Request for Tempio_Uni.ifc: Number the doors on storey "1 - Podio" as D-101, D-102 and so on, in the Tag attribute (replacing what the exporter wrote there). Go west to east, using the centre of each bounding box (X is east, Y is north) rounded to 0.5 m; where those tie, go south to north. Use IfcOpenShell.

First a look at what the model holds.

```python
import ifcopenshell
import ifcopenshell.util.element
import ifcopenshell.util.placement

model = ifcopenshell.open("Tempio_Uni.ifc")
print(model.schema)
storey = next(s for s in model.by_type("IfcBuildingStorey") if s.Name == "1 - Podio")
doors = [e for e in ifcopenshell.util.element.get_decomposition(storey) if e.is_a("IfcDoor")]
for e in sorted(doors, key=lambda e: e.id()):
    origin = ifcopenshell.util.placement.get_local_placement(e.ObjectPlacement)[:3, 3]
    print(e.id(), e.Tag, e.Name, origin.round(2) + 0.0, sep=" | ")
```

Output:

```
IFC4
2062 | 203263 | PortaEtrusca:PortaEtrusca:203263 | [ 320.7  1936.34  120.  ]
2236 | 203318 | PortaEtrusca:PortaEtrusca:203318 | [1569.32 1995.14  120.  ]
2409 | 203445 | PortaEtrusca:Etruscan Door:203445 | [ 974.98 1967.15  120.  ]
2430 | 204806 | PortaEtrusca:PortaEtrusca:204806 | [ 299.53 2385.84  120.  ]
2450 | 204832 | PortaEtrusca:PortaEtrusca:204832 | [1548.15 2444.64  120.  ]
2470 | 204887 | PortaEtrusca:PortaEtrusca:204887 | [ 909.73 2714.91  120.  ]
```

```python
import ifcopenshell
import ifcopenshell.geom
import ifcopenshell.util.element
import ifcopenshell.util.shape

model = ifcopenshell.open("Tempio_Uni.ifc")
settings = ifcopenshell.geom.settings()
settings.set("use-world-coords", True)


def centre(element):
    shape = ifcopenshell.geom.create_shape(settings, element)
    return ifcopenshell.util.shape.get_bbox_centroid(shape.geometry)


storey = next(s for s in model.by_type("IfcBuildingStorey") if s.Name == "1 - Podio")
doors = [e for e in ifcopenshell.util.element.get_decomposition(storey) if e.is_a("IfcDoor")]

# Insertion points can sit at a corner or the storey origin, so sort by the geometry (in metres).
centres = {e: centre(e) for e in doors}
doors.sort(key=lambda e: (round(centres[e][0] / 0.5), centres[e][1]))

for i, e in enumerate(doors, start=1):
    number = f"D-1{i:02d}"
    e.Tag = number
    print(e.id(), number)

model.write("Tempio_Uni_v2.ifc")
```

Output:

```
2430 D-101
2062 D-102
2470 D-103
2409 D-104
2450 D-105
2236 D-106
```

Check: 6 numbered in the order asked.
